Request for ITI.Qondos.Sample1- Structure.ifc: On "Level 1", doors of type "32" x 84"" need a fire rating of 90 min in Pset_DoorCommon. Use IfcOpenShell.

First a look at what the model holds.

```python
import ifcopenshell
import ifcopenshell.util.element

model = ifcopenshell.open("ITI.Qondos.Sample1- Structure.ifc")
print(model.schema)
storey = next(s for s in model.by_type("IfcBuildingStorey") if s.Name == "Level 1")
doors = [e for e in ifcopenshell.util.element.get_decomposition(storey) if e.is_a("IfcDoor")]
seen = {}
for e in doors:
    element_type = ifcopenshell.util.element.get_type(e)
    key = (element_type.Name if element_type != e and element_type else None, ifcopenshell.util.element.get_pset(e, "Pset_DoorCommon", "FireRating"))
    seen[key] = seen.get(key, 0) + 1
for (name, value), count in sorted(seen.items(), key=str):
    print(count, "x", name, "|", value)
```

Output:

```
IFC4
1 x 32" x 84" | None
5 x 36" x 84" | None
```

```python
import ifcopenshell
import ifcopenshell.api.pset
import ifcopenshell.util.element

model = ifcopenshell.open("ITI.Qondos.Sample1- Structure.ifc")

storey = next(s for s in model.by_type("IfcBuildingStorey") if s.Name == "Level 1")
doors = [e for e in ifcopenshell.util.element.get_decomposition(storey) if e.is_a("IfcDoor")]

count = 0
for e in doors:
    element_type = ifcopenshell.util.element.get_type(e)
    if element_type in (None, e) or element_type.Name != '32" x 84"':
        continue
    # add_pset returns the element's existing set when there is one.
    pset = ifcopenshell.api.pset.add_pset(model, product=e, name="Pset_DoorCommon")
    ifcopenshell.api.pset.edit_pset(model, pset=pset, properties={"FireRating": "90 min"})
    count += 1

print(count, "doors updated")

model.write("ITI.Qondos.Sample1- Structure_updated.ifc")
```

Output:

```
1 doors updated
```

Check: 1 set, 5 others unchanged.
